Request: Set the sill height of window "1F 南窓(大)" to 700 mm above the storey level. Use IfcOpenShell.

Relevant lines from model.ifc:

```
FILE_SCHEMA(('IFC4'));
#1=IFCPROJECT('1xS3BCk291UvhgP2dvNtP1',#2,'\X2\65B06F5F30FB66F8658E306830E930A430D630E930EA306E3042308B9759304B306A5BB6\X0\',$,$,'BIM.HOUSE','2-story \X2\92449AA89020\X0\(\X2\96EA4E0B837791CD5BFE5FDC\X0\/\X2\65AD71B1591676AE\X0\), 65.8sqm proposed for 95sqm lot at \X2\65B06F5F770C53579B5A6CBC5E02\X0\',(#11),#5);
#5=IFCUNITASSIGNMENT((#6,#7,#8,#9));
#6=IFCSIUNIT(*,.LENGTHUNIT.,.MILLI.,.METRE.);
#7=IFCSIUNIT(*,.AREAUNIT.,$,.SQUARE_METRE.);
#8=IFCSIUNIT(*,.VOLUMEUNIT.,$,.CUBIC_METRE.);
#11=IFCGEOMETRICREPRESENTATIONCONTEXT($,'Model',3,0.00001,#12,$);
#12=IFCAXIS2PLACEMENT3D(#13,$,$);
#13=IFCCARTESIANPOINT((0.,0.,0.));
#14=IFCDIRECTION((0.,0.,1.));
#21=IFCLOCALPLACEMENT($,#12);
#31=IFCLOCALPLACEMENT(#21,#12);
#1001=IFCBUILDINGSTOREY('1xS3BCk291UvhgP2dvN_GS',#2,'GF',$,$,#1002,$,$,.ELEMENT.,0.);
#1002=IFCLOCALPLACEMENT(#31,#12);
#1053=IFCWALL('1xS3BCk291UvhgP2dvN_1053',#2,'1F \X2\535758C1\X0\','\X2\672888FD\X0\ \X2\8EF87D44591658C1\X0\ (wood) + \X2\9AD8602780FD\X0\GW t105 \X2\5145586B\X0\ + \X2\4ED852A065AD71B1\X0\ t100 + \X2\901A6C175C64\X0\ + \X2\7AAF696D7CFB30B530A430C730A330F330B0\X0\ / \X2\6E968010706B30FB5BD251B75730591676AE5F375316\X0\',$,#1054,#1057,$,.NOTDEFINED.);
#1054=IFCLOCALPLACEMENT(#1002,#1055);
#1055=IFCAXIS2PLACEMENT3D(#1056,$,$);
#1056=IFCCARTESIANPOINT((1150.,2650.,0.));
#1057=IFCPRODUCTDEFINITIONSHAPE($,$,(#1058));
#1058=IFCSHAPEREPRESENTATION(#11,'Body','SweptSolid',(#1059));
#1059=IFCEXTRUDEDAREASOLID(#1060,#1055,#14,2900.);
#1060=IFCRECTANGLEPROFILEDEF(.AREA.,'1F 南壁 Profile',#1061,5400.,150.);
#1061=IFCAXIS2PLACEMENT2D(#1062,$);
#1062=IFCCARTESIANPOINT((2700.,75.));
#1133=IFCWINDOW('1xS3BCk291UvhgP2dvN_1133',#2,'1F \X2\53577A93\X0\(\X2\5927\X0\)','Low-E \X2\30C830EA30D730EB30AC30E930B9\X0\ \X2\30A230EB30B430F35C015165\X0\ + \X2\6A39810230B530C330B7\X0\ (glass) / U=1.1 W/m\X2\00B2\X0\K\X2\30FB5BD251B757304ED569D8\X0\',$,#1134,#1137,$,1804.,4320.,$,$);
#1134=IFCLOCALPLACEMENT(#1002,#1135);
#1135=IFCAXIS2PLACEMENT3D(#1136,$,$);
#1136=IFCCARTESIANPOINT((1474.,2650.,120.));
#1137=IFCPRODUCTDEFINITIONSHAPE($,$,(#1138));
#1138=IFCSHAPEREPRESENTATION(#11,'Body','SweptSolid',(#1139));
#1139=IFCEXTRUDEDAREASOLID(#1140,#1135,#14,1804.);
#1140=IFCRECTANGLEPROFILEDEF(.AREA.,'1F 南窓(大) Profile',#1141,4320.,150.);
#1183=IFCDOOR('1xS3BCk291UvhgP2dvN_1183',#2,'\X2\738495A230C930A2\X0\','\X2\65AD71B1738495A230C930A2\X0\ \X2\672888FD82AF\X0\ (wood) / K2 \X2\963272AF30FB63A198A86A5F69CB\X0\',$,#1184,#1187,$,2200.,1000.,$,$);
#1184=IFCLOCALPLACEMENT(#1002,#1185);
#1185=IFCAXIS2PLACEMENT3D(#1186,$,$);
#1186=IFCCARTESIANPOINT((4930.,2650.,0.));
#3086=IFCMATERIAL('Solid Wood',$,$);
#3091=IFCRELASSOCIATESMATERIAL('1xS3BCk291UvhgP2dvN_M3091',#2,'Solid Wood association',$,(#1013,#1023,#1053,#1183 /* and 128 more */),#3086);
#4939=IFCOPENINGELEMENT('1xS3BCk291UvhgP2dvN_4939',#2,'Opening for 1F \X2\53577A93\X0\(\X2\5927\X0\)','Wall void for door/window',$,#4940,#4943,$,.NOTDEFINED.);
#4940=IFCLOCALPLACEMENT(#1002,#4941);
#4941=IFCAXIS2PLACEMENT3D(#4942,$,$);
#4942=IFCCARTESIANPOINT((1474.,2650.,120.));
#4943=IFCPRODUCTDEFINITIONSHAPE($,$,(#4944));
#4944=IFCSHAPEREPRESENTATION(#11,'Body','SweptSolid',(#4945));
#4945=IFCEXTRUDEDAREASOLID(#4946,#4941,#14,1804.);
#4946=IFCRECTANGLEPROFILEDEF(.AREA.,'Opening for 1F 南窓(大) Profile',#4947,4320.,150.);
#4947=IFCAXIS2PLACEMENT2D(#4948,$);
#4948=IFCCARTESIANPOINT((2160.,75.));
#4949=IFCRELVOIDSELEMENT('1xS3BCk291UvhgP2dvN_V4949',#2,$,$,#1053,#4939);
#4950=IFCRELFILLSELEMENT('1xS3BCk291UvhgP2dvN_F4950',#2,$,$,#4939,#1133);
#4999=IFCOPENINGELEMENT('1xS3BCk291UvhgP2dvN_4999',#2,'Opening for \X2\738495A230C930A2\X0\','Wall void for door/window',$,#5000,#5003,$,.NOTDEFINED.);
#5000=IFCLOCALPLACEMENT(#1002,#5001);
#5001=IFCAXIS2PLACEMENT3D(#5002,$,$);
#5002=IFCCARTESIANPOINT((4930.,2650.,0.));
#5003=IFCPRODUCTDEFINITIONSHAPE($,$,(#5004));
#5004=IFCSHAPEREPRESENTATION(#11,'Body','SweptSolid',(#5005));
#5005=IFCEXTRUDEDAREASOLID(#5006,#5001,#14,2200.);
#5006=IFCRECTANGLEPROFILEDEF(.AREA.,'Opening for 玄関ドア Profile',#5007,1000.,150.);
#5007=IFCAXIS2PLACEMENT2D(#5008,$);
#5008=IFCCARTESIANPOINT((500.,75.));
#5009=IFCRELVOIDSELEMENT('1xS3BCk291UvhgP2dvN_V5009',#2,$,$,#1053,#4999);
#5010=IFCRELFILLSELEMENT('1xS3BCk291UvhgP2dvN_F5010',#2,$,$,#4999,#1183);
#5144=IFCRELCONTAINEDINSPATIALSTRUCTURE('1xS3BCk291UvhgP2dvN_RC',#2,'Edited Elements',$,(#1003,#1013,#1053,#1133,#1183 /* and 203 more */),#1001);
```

```python
import numpy as np
import ifcopenshell
import ifcopenshell.api.geometry
import ifcopenshell.geom
import ifcopenshell.util.element
import ifcopenshell.util.placement
import ifcopenshell.util.shape
import ifcopenshell.util.unit

model = ifcopenshell.open("model.ifc")
unit_scale = ifcopenshell.util.unit.calculate_unit_scale(model)

window = model.by_id(1133)
opening = window.FillsVoids[0].RelatingOpeningElement
storey = ifcopenshell.util.element.get_container(window, ifc_class="IfcBuildingStorey")
level = ifcopenshell.util.placement.get_local_placement(storey.ObjectPlacement)[2, 3]

# The opening's origin need not be at the sill, so measure its lowest point.
shape = ifcopenshell.geom.create_shape(ifcopenshell.geom.settings(), opening)
bottom = ifcopenshell.util.shape.get_shape_bottom_elevation(shape, shape.geometry) / unit_scale
dz = level + 0.7 / unit_scale - bottom

shift = np.array([0.0, 0.0, dz])
# The window is not placed relative to its opening, so move both.
for product in (opening, window):
    matrix = ifcopenshell.util.placement.get_local_placement(product.ObjectPlacement)
    matrix[:3, 3] += shift
    ifcopenshell.api.geometry.edit_object_placement(model, product=product, matrix=matrix, is_si=False)

print(f"moved by {dz * unit_scale:+.3f} m")

model.write("model_rev.ifc")
```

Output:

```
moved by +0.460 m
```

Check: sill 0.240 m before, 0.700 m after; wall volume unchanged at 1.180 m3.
